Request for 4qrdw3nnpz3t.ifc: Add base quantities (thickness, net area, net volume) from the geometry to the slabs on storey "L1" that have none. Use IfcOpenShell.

First a look at what the model holds.

```python
import ifcopenshell
import ifcopenshell.util.element
import ifcopenshell.util.unit

model = ifcopenshell.open("4qrdw3nnpz3t.ifc")
print(model.schema)
for unit_type in ("LENGTHUNIT", "AREAUNIT", "VOLUMEUNIT"):
    print(unit_type, ifcopenshell.util.unit.calculate_unit_scale(model, unit_type))
storey = next(s for s in model.by_type("IfcBuildingStorey") if s.Name == "L1")
slabs = [e for e in ifcopenshell.util.element.get_decomposition(storey) if e.is_a("IfcSlab")]
for e in sorted(slabs, key=lambda e: e.id()):
    print(e.id(), e.is_a(), e.Name, list(ifcopenshell.util.element.get_psets(e, qtos_only=True)), sep=" | ")
```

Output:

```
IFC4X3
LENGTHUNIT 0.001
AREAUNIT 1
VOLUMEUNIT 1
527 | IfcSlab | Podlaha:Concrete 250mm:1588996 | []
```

```python
import ifcopenshell
import ifcopenshell.api.pset
import ifcopenshell.geom
import ifcopenshell.util.element
import ifcopenshell.util.shape
import ifcopenshell.util.unit

model = ifcopenshell.open("4qrdw3nnpz3t.ifc")
unit_scale = ifcopenshell.util.unit.calculate_unit_scale(model)
area_scale = ifcopenshell.util.unit.calculate_unit_scale(model, "AREAUNIT")
volume_scale = ifcopenshell.util.unit.calculate_unit_scale(model, "VOLUMEUNIT")
settings = ifcopenshell.geom.settings()

storey = next(s for s in model.by_type("IfcBuildingStorey") if s.Name == "L1")
slabs = [e for e in ifcopenshell.util.element.get_decomposition(storey) if e.is_a("IfcSlab")]

for e in sorted(slabs, key=lambda e: e.id()):
    if ifcopenshell.util.element.get_psets(e, qtos_only=True, should_inherit=False):
        continue
    # Geometry comes back in metres, in the element's own axes.
    shape = ifcopenshell.geom.create_shape(settings, e)
    values = {
        "Width": ifcopenshell.util.shape.get_z(shape.geometry) / unit_scale,
        "NetArea": ifcopenshell.util.shape.get_footprint_area(shape.geometry) / area_scale,
        "NetVolume": ifcopenshell.util.shape.get_volume(shape.geometry) / volume_scale,
    }
    qto = ifcopenshell.api.pset.add_qto(model, product=e, name="Qto_SlabBaseQuantities")
    ifcopenshell.api.pset.edit_qto(model, qto=qto, properties=values)
    print(e.id(), {k: round(v, 3) for k, v in values.items()})

model.write("4qrdw3nnpz3t-out.ifc")
```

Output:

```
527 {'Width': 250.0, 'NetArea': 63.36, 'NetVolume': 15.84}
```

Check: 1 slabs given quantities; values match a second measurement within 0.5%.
